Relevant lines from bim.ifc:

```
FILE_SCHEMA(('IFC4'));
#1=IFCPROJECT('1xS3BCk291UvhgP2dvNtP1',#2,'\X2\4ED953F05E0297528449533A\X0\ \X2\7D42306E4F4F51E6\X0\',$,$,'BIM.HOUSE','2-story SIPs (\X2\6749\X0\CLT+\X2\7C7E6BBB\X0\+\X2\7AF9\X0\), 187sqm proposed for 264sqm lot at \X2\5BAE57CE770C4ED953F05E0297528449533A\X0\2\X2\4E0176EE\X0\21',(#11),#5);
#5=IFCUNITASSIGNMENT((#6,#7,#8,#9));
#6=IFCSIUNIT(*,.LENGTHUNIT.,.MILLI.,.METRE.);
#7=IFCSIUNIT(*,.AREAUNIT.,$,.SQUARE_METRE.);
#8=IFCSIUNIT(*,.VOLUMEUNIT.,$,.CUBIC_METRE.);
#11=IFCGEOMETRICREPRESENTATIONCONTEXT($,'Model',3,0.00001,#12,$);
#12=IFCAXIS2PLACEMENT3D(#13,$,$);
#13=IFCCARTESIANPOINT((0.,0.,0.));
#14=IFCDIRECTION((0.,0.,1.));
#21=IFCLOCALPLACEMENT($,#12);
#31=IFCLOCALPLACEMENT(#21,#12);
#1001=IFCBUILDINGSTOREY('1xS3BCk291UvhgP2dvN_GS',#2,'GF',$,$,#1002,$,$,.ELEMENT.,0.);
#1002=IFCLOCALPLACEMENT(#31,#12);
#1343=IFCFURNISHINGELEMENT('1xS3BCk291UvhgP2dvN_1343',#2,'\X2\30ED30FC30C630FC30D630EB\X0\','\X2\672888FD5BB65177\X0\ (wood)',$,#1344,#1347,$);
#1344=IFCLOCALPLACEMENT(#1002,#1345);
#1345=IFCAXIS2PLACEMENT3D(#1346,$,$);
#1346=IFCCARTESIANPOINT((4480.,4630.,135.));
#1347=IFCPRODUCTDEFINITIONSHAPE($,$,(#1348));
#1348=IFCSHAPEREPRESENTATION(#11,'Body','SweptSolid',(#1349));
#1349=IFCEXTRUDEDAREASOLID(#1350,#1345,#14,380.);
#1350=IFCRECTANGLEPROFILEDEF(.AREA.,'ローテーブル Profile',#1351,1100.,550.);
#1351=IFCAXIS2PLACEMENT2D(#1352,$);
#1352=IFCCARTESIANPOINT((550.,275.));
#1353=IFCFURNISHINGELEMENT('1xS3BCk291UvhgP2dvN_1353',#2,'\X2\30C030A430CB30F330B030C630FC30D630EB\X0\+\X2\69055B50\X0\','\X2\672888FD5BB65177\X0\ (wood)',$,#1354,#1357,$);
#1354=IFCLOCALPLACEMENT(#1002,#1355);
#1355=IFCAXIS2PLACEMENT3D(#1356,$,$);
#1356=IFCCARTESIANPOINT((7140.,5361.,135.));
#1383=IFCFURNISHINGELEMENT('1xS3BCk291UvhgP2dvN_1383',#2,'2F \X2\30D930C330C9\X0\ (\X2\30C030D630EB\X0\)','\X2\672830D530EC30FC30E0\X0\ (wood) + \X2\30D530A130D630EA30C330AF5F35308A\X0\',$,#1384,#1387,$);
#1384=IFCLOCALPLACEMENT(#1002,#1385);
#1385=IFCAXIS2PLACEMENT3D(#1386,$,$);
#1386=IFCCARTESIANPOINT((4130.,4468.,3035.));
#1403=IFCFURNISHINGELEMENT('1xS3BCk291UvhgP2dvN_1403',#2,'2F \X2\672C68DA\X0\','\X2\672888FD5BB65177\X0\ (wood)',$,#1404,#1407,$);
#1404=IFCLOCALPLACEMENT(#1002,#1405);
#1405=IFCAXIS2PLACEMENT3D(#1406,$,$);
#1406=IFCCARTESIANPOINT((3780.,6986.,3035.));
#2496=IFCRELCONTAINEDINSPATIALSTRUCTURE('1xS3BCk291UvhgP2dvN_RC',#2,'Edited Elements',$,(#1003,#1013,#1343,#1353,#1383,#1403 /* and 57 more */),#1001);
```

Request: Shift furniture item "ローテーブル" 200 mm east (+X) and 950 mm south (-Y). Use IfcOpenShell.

```python
import ifcopenshell
import ifcopenshell.api.geometry
import ifcopenshell.util.placement
import ifcopenshell.util.unit

model = ifcopenshell.open("bim.ifc")
unit_scale = ifcopenshell.util.unit.calculate_unit_scale(model)

item = model.by_guid("1xS3BCk291UvhgP2dvN_1343")
matrix = ifcopenshell.util.placement.get_local_placement(item.ObjectPlacement)
matrix[0, 3] += 0.2 / unit_scale
matrix[1, 3] -= 0.95 / unit_scale
ifcopenshell.api.geometry.edit_object_placement(model, product=item, matrix=matrix, is_si=False)

print(ifcopenshell.util.placement.get_local_placement(item.ObjectPlacement).round(3) + 0.0)

model.write("bim_rev.ifc")
```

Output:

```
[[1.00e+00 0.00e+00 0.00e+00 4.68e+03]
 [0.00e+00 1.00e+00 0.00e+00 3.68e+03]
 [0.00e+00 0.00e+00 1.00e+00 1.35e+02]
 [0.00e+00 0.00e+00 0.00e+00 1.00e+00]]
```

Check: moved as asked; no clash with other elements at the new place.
